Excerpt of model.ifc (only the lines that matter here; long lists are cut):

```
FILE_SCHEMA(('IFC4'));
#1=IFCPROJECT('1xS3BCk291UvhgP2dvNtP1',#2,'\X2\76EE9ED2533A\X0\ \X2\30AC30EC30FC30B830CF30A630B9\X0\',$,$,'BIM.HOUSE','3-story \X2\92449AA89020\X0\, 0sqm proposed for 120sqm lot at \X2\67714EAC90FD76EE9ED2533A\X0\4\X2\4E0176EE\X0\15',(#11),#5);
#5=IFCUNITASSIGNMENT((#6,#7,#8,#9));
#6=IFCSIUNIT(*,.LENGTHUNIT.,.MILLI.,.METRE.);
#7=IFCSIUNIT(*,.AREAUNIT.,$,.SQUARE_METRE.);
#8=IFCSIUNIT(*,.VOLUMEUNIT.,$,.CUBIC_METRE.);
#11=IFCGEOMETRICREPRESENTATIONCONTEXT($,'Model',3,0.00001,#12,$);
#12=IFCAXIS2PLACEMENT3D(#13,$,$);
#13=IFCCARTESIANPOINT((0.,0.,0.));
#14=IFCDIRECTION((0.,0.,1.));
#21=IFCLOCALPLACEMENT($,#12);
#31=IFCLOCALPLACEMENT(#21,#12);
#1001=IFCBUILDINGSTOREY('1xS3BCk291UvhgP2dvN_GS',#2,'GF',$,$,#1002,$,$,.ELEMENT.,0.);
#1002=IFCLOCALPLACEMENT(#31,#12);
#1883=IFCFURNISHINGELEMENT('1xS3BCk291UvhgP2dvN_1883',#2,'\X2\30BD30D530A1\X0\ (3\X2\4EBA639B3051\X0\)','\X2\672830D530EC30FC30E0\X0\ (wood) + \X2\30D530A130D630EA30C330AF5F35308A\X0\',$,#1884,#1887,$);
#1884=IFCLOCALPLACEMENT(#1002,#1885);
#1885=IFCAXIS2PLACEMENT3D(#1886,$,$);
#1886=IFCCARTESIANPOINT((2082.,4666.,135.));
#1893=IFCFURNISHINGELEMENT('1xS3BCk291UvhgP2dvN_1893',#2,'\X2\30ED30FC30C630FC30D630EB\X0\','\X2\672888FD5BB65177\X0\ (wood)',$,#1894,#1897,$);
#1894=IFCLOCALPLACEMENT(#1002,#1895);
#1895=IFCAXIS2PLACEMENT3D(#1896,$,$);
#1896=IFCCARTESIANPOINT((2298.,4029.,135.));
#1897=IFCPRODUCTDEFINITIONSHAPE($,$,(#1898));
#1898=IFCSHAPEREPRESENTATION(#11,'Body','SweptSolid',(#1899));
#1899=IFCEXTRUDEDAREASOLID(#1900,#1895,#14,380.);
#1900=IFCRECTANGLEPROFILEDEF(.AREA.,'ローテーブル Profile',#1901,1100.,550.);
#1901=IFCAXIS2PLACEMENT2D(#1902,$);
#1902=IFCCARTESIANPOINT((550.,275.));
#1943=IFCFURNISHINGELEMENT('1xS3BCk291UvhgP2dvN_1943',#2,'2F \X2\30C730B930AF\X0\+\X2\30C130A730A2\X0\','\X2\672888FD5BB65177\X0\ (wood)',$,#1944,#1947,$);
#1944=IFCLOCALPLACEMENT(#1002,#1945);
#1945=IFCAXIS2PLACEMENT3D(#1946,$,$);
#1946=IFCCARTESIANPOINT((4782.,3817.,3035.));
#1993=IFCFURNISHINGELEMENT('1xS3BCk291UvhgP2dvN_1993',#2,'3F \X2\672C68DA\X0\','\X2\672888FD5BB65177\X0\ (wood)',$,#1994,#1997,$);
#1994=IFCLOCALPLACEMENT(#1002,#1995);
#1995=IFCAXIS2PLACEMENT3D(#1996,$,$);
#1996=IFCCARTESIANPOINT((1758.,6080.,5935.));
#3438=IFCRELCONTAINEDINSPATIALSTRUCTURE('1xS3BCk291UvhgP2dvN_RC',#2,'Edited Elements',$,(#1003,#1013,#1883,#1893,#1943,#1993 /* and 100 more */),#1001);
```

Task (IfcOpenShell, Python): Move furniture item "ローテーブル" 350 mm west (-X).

```python
import ifcopenshell
import ifcopenshell.api.geometry
import ifcopenshell.util.placement
import ifcopenshell.util.unit

model = ifcopenshell.open("model.ifc")
unit_scale = ifcopenshell.util.unit.calculate_unit_scale(model)

item = model.by_guid("1xS3BCk291UvhgP2dvN_1893")
matrix = ifcopenshell.util.placement.get_local_placement(item.ObjectPlacement)
matrix[0, 3] -= 0.35 / unit_scale
ifcopenshell.api.geometry.edit_object_placement(model, product=item, matrix=matrix, is_si=False)

print(ifcopenshell.util.placement.get_local_placement(item.ObjectPlacement).round(3) + 0.0)

model.write("model_updated.ifc")
```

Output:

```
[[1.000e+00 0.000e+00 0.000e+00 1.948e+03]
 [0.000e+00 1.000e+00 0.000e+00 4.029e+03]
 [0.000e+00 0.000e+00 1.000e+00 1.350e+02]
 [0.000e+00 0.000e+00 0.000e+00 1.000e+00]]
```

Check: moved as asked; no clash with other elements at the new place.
